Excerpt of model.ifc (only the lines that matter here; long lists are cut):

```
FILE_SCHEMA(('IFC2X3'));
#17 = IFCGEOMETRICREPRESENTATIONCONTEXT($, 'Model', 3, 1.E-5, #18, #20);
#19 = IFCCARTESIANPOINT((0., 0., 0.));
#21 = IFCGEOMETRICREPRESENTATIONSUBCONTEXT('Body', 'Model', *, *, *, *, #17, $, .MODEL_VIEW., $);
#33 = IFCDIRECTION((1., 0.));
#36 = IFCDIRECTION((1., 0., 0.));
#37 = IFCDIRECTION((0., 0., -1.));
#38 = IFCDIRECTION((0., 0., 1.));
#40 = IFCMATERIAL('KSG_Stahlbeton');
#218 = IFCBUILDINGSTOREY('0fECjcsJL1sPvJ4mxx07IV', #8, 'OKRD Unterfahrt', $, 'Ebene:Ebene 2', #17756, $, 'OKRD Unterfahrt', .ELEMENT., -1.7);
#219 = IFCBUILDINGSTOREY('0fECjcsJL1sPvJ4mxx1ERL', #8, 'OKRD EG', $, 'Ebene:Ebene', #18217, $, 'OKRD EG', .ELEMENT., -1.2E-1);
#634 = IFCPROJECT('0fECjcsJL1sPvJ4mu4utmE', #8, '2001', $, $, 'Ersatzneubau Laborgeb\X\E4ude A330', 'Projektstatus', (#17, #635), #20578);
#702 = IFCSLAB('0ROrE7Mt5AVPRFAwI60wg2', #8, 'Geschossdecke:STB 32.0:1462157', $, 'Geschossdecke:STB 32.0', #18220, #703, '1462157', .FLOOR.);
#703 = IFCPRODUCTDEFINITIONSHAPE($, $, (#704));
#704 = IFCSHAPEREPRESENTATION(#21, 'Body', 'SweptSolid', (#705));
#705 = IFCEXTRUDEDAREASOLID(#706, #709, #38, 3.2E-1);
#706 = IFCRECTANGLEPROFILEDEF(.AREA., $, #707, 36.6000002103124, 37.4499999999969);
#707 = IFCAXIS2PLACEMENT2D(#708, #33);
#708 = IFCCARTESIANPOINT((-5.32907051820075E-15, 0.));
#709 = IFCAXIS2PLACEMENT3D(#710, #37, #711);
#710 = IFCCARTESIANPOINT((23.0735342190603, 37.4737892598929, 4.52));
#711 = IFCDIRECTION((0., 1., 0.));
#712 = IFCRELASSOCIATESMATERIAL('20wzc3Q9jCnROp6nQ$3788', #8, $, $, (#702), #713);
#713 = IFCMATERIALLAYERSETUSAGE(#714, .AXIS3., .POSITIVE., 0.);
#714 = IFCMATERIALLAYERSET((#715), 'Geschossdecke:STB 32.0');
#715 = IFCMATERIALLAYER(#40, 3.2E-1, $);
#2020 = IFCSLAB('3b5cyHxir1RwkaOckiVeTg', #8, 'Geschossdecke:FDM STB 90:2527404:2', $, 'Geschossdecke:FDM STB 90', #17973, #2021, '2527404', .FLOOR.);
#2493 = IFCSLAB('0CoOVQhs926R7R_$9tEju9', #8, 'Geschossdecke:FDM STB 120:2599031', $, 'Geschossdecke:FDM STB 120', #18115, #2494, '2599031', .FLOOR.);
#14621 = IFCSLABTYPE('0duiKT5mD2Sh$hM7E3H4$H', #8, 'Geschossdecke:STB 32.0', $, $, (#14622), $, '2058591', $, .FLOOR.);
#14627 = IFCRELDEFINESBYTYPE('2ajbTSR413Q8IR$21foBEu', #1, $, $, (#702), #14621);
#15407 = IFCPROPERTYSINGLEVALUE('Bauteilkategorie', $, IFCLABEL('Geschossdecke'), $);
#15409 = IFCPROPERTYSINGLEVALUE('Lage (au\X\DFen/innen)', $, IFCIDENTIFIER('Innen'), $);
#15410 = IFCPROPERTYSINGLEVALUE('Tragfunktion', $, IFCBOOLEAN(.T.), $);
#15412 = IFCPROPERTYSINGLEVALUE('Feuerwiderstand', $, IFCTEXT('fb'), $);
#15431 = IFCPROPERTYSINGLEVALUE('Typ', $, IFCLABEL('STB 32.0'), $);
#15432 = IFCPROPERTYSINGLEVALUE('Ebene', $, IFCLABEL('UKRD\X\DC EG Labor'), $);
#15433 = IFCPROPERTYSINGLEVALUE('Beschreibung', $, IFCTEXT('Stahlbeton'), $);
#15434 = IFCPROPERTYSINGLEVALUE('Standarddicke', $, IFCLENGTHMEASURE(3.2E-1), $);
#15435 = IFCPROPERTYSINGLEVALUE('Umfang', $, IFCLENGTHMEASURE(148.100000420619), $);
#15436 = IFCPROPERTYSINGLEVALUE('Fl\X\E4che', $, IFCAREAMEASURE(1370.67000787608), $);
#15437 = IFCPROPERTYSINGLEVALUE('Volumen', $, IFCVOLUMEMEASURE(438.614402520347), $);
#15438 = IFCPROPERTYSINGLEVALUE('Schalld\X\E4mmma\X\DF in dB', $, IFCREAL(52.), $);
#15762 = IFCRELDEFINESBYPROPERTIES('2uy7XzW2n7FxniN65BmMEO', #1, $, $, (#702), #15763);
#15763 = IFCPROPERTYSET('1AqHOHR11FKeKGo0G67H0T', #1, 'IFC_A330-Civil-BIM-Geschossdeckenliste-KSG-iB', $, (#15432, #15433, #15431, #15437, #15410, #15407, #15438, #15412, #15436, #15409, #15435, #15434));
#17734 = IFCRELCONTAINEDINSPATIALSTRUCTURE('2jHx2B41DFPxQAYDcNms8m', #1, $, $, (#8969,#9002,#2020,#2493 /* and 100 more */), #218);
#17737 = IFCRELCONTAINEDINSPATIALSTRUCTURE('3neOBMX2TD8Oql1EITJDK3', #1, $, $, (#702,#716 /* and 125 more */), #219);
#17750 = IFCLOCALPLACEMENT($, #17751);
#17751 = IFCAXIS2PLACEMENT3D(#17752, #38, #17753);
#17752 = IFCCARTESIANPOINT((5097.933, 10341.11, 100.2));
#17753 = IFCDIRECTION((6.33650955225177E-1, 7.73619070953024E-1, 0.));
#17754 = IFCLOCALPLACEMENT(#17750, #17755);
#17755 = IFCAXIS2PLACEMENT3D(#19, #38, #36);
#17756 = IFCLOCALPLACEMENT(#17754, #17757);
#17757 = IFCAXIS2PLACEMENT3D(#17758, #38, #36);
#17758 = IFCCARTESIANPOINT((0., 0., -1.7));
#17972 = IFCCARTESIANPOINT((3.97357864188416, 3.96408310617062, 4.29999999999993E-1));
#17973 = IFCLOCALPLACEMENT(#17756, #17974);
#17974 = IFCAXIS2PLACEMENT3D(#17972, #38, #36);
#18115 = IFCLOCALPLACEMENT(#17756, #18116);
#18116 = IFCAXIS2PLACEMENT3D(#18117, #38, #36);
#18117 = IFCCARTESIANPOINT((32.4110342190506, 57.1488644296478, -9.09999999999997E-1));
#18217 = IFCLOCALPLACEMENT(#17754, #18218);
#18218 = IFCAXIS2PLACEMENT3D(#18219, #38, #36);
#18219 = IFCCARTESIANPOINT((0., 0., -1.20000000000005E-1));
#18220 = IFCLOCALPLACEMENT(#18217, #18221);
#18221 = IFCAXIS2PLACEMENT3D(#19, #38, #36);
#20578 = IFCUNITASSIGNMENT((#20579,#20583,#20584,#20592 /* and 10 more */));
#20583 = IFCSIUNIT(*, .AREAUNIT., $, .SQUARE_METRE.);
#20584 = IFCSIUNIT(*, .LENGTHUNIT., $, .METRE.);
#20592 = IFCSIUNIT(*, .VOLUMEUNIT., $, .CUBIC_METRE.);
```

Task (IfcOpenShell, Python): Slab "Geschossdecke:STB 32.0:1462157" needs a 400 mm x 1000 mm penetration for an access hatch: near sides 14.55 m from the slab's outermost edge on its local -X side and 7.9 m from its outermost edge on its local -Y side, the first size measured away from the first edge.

```python
import numpy as np
import ifcopenshell
import ifcopenshell.api.feature
import ifcopenshell.api.geometry
import ifcopenshell.api.pset
import ifcopenshell.api.root
import ifcopenshell.geom
import ifcopenshell.util.element
import ifcopenshell.util.placement
import ifcopenshell.util.representation
import ifcopenshell.util.shape
import ifcopenshell.util.unit

model = ifcopenshell.open("model.ifc")
unit_scale = ifcopenshell.util.unit.calculate_unit_scale(model)
area_scale = ifcopenshell.util.unit.calculate_unit_scale(model, "AREAUNIT")
volume_scale = ifcopenshell.util.unit.calculate_unit_scale(model, "VOLUMEUNIT")
settings = ifcopenshell.geom.settings()


def volume(element):
    """Net volume in cubic metres, openings subtracted."""
    shape = ifcopenshell.geom.create_shape(settings, element)
    return ifcopenshell.util.shape.get_volume(shape.geometry)


slab = model.by_guid("0ROrE7Mt5AVPRFAwI60wg2")
before = volume(slab)

# Extent in the slab's own axes, in metres. The edges named are its -X and -Y sides.
slab_shape = ifcopenshell.geom.create_shape(settings, slab)
vertices = ifcopenshell.util.shape.get_vertices(slab_shape.geometry)
x_min, y_min, bottom = vertices.min(axis=0)
top = vertices[:, 2].max()

opening = ifcopenshell.api.root.create_entity(model, ifc_class="IfcOpeningElement", name="Access hatch opening")
context = ifcopenshell.util.representation.get_context(model, "Model", "Body", "MODEL_VIEW")
width, depth = 0.4, 1
outline = [(0.0, 0.0), (width, 0.0), (width, depth), (0.0, depth), (0.0, 0.0)]
# Overshoot both faces by 50 mm so the cut is clean.
shape = ifcopenshell.api.geometry.add_slab_representation(
    model, context=context, depth=top - bottom + 0.1, polyline=outline
)
ifcopenshell.api.geometry.assign_representation(model, product=opening, representation=shape)

matrix = ifcopenshell.util.placement.get_local_placement(slab.ObjectPlacement)
matrix[:, 3] = matrix @ np.append(np.array([x_min + 14.55, y_min + 7.9, bottom - 0.05]) / unit_scale, 1.0)
ifcopenshell.api.geometry.edit_object_placement(model, product=opening, matrix=matrix, is_si=False)
ifcopenshell.api.feature.add_feature(model, feature=opening, element=slab)

after = volume(slab)

# Update the slab's stored quantities.
pset = model.by_id(ifcopenshell.util.element.get_pset(slab, "IFC_A330-Civil-BIM-Geschossdeckenliste-KSG-iB", should_inherit=False)["id"])
ifcopenshell.api.pset.edit_pset(model, pset=pset, properties={
    "Volumen": model.create_entity("IfcVolumeMeasure", after / volume_scale),
    "Fläche": model.create_entity("IfcAreaMeasure", after / (top - bottom) / area_scale),
})

print(f"slab volume {before:.3f} -> {after:.3f} m3")

model.write("model_edited.ifc")
```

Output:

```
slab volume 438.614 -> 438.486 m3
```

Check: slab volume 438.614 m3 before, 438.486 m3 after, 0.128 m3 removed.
